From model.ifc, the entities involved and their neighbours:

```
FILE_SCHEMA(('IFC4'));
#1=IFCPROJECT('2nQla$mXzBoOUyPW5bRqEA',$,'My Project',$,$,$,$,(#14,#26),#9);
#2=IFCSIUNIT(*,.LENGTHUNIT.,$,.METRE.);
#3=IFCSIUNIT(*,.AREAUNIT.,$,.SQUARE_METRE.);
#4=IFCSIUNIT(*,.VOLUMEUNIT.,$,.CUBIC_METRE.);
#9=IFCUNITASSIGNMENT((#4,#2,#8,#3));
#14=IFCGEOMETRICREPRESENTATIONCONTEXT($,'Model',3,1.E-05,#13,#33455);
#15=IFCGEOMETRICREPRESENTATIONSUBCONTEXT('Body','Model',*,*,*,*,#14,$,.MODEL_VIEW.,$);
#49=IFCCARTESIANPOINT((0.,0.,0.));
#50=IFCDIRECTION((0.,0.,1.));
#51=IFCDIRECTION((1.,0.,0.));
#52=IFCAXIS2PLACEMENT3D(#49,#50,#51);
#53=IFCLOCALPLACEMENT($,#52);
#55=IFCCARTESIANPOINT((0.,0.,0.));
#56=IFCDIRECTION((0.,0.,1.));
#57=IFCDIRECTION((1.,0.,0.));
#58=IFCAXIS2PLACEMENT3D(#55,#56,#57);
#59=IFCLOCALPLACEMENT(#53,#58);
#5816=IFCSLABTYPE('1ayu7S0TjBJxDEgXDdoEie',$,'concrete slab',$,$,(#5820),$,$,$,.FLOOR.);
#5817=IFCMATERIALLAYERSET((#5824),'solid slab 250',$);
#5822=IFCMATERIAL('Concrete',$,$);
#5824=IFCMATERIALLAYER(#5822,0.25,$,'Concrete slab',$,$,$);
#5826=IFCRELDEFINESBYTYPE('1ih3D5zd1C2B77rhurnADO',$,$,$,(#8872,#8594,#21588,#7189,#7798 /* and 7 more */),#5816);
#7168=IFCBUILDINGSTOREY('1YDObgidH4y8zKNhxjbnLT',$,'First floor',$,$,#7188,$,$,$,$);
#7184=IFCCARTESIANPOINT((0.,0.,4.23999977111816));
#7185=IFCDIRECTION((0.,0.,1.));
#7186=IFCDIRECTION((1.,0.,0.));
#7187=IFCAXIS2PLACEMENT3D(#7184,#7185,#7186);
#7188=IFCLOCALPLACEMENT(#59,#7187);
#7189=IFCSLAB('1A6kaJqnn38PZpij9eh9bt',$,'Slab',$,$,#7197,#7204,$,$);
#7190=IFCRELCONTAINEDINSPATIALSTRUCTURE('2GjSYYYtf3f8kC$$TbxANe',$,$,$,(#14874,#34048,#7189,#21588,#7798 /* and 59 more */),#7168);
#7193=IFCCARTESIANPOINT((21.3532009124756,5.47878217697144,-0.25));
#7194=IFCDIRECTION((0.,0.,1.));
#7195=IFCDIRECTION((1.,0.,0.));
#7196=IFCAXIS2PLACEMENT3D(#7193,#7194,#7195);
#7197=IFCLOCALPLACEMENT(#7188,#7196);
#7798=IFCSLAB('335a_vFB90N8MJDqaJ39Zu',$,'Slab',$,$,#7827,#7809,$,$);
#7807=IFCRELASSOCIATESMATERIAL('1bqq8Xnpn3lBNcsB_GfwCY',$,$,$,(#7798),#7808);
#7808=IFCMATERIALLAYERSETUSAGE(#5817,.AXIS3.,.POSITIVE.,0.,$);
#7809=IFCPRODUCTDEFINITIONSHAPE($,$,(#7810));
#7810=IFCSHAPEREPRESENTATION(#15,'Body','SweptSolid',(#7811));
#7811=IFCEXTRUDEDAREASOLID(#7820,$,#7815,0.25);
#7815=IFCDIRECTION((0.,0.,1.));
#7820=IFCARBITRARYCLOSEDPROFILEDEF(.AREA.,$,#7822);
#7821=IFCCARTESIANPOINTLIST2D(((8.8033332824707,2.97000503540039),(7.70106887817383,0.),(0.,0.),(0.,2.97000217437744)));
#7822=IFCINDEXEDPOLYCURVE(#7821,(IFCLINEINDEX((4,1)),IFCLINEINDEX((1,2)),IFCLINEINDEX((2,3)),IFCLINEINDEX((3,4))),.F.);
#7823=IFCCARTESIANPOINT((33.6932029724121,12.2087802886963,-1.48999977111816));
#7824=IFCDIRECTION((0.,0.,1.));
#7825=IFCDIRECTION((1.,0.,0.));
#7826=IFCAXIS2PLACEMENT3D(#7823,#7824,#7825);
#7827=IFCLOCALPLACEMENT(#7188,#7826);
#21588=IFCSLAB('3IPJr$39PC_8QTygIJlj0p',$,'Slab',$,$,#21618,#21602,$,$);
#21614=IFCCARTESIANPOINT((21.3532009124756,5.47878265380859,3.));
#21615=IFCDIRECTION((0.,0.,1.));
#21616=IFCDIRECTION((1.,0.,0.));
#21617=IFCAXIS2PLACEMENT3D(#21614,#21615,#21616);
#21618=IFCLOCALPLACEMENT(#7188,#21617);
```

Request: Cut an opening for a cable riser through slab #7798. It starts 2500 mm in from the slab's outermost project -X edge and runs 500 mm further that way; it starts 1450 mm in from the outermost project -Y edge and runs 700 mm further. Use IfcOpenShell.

```python
import numpy as np
import ifcopenshell
import ifcopenshell.api.feature
import ifcopenshell.api.geometry
import ifcopenshell.api.root
import ifcopenshell.geom
import ifcopenshell.util.placement
import ifcopenshell.util.representation
import ifcopenshell.util.shape
import ifcopenshell.util.unit

model = ifcopenshell.open("model.ifc")
unit_scale = ifcopenshell.util.unit.calculate_unit_scale(model)
settings = ifcopenshell.geom.settings()


def volume(element):
    """Net volume in cubic metres, openings subtracted."""
    shape = ifcopenshell.geom.create_shape(settings, element)
    return ifcopenshell.util.shape.get_volume(shape.geometry)


slab = model.by_guid("335a_vFB90N8MJDqaJ39Zu")
before = volume(slab)

# Extent in the slab's own axes, in metres. The edges named are its -X and -Y sides.
slab_shape = ifcopenshell.geom.create_shape(settings, slab)
vertices = ifcopenshell.util.shape.get_vertices(slab_shape.geometry)
x_min, y_min, bottom = vertices.min(axis=0)
top = vertices[:, 2].max()

opening = ifcopenshell.api.root.create_entity(model, ifc_class="IfcOpeningElement", name="Cable riser opening", predefined_type="OPENING")
context = ifcopenshell.util.representation.get_context(model, "Model", "Body", "MODEL_VIEW")
width, depth = 0.5, 0.7
outline = [(0.0, 0.0), (width, 0.0), (width, depth), (0.0, depth), (0.0, 0.0)]
# Overshoot both faces by 50 mm so the cut is clean.
shape = ifcopenshell.api.geometry.add_slab_representation(
    model, context=context, depth=top - bottom + 0.1, polyline=outline
)
ifcopenshell.api.geometry.assign_representation(model, product=opening, representation=shape)

matrix = ifcopenshell.util.placement.get_local_placement(slab.ObjectPlacement)
matrix[:, 3] = matrix @ np.append(np.array([x_min + 2.5, y_min + 1.45, bottom - 0.05]) / unit_scale, 1.0)
ifcopenshell.api.geometry.edit_object_placement(model, product=opening, matrix=matrix, is_si=False)
ifcopenshell.api.feature.add_feature(model, feature=opening, element=slab)

after = volume(slab)

print(f"slab volume {before:.3f} -> {after:.3f} m3")

model.write("model_edited.ifc")
```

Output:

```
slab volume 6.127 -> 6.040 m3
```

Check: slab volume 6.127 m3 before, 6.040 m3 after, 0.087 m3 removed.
